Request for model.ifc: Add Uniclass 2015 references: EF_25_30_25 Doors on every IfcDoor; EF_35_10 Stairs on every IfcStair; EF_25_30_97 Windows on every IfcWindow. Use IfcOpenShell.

First a look at what the model holds.

```python
import ifcopenshell

model = ifcopenshell.open("model.ifc")
print(model.schema)
print("classifications:", [c.Name for c in model.by_type("IfcClassification")])
for ifc_class in ("IfcDoor", "IfcRoof", "IfcStair", "IfcWall", "IfcWindow"):
    print(ifc_class, len(model.by_type(ifc_class)))
```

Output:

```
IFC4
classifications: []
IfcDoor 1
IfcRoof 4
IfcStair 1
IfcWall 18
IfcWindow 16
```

```python
import ifcopenshell
import ifcopenshell.api.classification

model = ifcopenshell.open("model.ifc")

system = ifcopenshell.api.classification.add_classification(model, classification="Uniclass 2015")

codes = {
    "IfcDoor": ("EF_25_30_25", "Doors"),
    "IfcStair": ("EF_35_10", "Stairs"),
    "IfcWindow": ("EF_25_30_97", "Windows"),
}
for ifc_class, (code, name) in codes.items():
    products = model.by_type(ifc_class)
    ifcopenshell.api.classification.add_reference(
        model, products=products, classification=system, identification=code, name=name
    )
    print(code, len(products))

model.write("model_v2.ifc")
```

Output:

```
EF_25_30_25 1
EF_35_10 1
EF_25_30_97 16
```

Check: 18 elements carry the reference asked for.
